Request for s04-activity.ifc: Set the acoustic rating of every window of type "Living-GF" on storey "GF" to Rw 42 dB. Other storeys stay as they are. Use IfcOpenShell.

First a look at what the model holds.

```python
import ifcopenshell
import ifcopenshell.util.element

model = ifcopenshell.open("s04-activity.ifc")
print(model.schema)
storey = next(s for s in model.by_type("IfcBuildingStorey") if s.Name == "GF")
windows = [e for e in ifcopenshell.util.element.get_decomposition(storey) if e.is_a("IfcWindow")]
seen = {}
for e in windows:
    element_type = ifcopenshell.util.element.get_type(e)
    key = (element_type.Name if element_type != e and element_type else None, ifcopenshell.util.element.get_pset(e, "Pset_WindowCommon", "AcousticRating"))
    seen[key] = seen.get(key, 0) + 1
for (name, value), count in sorted(seen.items(), key=str):
    print(count, "x", name, "|", value)
```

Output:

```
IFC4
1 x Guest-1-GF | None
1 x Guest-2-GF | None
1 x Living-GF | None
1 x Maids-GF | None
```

```python
import ifcopenshell
import ifcopenshell.api.pset
import ifcopenshell.util.element

model = ifcopenshell.open("s04-activity.ifc")

storey = next(s for s in model.by_type("IfcBuildingStorey") if s.Name == "GF")
windows = [e for e in ifcopenshell.util.element.get_decomposition(storey) if e.is_a("IfcWindow")]

count = 0
for e in windows:
    element_type = ifcopenshell.util.element.get_type(e)
    if element_type in (None, e) or element_type.Name != "Living-GF":
        continue
    # add_pset returns the element's existing set when there is one.
    pset = ifcopenshell.api.pset.add_pset(model, product=e, name="Pset_WindowCommon")
    ifcopenshell.api.pset.edit_pset(model, pset=pset, properties={"AcousticRating": "Rw 42 dB"})
    count += 1

print(count, "windows updated")

model.write("s04-activity_v2.ifc")
```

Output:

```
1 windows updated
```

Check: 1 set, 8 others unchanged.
